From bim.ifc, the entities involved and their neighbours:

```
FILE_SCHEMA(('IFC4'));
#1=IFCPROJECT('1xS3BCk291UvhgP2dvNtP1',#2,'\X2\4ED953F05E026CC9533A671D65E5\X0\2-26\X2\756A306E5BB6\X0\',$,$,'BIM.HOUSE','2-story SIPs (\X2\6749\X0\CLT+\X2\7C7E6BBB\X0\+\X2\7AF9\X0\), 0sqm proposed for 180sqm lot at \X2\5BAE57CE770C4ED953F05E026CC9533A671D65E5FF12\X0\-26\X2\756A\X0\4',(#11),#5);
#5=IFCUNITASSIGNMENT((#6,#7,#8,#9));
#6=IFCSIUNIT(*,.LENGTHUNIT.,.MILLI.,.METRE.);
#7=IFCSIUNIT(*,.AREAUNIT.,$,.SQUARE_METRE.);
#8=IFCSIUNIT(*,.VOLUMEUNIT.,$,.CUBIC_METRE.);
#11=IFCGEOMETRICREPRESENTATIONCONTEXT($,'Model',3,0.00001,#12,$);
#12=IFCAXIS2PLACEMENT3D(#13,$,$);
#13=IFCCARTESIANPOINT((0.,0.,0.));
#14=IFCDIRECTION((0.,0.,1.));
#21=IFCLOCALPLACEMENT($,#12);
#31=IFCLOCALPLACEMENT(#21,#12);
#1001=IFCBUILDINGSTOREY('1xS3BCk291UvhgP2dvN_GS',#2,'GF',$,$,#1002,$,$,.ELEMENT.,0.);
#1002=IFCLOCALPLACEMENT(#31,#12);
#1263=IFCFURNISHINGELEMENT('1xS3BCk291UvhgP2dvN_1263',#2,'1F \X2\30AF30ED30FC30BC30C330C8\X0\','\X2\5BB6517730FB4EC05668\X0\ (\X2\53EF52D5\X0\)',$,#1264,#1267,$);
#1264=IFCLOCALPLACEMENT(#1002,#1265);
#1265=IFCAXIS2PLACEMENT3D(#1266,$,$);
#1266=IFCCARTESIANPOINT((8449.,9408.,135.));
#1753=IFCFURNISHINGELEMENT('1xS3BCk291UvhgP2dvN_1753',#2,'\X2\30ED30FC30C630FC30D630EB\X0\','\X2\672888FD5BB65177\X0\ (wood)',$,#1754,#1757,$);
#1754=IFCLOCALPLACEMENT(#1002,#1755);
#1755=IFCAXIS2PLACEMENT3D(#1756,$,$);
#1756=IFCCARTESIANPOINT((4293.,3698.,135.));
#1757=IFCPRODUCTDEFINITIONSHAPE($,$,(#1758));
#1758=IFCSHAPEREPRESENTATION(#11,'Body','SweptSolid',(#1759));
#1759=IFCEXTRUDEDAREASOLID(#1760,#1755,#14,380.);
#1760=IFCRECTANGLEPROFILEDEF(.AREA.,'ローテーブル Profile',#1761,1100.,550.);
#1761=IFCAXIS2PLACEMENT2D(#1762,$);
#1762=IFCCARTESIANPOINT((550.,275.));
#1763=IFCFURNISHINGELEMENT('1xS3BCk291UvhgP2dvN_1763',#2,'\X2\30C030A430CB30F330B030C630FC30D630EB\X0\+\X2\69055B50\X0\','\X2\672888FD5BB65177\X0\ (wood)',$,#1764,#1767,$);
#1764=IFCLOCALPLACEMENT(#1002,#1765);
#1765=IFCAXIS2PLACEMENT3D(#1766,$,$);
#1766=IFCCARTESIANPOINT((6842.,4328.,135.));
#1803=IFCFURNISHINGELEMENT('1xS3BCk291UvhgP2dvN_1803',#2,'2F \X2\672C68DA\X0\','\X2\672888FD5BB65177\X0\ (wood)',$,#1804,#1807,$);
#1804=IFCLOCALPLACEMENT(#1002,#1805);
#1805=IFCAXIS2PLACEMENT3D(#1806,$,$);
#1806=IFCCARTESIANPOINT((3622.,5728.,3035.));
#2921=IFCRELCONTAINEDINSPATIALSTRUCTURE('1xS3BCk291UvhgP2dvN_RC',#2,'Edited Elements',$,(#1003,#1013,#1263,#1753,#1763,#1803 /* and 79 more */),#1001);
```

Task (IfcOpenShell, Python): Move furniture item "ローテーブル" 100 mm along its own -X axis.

```python
import ifcopenshell
import ifcopenshell.api.geometry
import ifcopenshell.util.placement
import ifcopenshell.util.unit

model = ifcopenshell.open("bim.ifc")
unit_scale = ifcopenshell.util.unit.calculate_unit_scale(model)

item = model.by_guid("1xS3BCk291UvhgP2dvN_1753")
matrix = ifcopenshell.util.placement.get_local_placement(item.ObjectPlacement)
matrix[:3, 3] -= matrix[:3, 0] * 0.1 / unit_scale
ifcopenshell.api.geometry.edit_object_placement(model, product=item, matrix=matrix, is_si=False)

print(ifcopenshell.util.placement.get_local_placement(item.ObjectPlacement).round(3) + 0.0)

model.write("bim_v2.ifc")
```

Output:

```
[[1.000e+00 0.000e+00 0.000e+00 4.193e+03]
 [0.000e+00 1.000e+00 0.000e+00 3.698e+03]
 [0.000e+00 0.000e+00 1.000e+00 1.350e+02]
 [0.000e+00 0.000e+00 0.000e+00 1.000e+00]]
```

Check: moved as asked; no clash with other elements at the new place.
